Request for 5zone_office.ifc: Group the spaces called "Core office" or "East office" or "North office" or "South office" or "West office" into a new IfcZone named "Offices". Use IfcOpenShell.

First a look at what the model holds.

```python
import ifcopenshell

model = ifcopenshell.open("5zone_office.ifc")
print(model.schema)
seen = {}
for space in model.by_type("IfcSpace"):
    seen[space.LongName] = seen.get(space.LongName, 0) + 1
for name, count in sorted(seen.items(), key=str):
    print(count, "x", name)
print("zones:", [z.Name for z in model.by_type("IfcZone")][:20])
```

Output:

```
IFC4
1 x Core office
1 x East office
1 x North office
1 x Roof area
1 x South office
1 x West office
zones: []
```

```python
import ifcopenshell
import ifcopenshell.api.group
import ifcopenshell.api.root

model = ifcopenshell.open("5zone_office.ifc")

names = {"Core office", "East office", "North office", "South office", "West office"}
spaces = [s for s in model.by_type("IfcSpace") if s.LongName in names]

zone = ifcopenshell.api.root.create_entity(model, ifc_class="IfcZone", name="Offices")
ifcopenshell.api.group.assign_group(model, products=spaces, group=zone)
print(len(spaces), "spaces in", zone.Name)

model.write("5zone_office_edited.ifc")
```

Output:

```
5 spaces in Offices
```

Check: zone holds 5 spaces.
